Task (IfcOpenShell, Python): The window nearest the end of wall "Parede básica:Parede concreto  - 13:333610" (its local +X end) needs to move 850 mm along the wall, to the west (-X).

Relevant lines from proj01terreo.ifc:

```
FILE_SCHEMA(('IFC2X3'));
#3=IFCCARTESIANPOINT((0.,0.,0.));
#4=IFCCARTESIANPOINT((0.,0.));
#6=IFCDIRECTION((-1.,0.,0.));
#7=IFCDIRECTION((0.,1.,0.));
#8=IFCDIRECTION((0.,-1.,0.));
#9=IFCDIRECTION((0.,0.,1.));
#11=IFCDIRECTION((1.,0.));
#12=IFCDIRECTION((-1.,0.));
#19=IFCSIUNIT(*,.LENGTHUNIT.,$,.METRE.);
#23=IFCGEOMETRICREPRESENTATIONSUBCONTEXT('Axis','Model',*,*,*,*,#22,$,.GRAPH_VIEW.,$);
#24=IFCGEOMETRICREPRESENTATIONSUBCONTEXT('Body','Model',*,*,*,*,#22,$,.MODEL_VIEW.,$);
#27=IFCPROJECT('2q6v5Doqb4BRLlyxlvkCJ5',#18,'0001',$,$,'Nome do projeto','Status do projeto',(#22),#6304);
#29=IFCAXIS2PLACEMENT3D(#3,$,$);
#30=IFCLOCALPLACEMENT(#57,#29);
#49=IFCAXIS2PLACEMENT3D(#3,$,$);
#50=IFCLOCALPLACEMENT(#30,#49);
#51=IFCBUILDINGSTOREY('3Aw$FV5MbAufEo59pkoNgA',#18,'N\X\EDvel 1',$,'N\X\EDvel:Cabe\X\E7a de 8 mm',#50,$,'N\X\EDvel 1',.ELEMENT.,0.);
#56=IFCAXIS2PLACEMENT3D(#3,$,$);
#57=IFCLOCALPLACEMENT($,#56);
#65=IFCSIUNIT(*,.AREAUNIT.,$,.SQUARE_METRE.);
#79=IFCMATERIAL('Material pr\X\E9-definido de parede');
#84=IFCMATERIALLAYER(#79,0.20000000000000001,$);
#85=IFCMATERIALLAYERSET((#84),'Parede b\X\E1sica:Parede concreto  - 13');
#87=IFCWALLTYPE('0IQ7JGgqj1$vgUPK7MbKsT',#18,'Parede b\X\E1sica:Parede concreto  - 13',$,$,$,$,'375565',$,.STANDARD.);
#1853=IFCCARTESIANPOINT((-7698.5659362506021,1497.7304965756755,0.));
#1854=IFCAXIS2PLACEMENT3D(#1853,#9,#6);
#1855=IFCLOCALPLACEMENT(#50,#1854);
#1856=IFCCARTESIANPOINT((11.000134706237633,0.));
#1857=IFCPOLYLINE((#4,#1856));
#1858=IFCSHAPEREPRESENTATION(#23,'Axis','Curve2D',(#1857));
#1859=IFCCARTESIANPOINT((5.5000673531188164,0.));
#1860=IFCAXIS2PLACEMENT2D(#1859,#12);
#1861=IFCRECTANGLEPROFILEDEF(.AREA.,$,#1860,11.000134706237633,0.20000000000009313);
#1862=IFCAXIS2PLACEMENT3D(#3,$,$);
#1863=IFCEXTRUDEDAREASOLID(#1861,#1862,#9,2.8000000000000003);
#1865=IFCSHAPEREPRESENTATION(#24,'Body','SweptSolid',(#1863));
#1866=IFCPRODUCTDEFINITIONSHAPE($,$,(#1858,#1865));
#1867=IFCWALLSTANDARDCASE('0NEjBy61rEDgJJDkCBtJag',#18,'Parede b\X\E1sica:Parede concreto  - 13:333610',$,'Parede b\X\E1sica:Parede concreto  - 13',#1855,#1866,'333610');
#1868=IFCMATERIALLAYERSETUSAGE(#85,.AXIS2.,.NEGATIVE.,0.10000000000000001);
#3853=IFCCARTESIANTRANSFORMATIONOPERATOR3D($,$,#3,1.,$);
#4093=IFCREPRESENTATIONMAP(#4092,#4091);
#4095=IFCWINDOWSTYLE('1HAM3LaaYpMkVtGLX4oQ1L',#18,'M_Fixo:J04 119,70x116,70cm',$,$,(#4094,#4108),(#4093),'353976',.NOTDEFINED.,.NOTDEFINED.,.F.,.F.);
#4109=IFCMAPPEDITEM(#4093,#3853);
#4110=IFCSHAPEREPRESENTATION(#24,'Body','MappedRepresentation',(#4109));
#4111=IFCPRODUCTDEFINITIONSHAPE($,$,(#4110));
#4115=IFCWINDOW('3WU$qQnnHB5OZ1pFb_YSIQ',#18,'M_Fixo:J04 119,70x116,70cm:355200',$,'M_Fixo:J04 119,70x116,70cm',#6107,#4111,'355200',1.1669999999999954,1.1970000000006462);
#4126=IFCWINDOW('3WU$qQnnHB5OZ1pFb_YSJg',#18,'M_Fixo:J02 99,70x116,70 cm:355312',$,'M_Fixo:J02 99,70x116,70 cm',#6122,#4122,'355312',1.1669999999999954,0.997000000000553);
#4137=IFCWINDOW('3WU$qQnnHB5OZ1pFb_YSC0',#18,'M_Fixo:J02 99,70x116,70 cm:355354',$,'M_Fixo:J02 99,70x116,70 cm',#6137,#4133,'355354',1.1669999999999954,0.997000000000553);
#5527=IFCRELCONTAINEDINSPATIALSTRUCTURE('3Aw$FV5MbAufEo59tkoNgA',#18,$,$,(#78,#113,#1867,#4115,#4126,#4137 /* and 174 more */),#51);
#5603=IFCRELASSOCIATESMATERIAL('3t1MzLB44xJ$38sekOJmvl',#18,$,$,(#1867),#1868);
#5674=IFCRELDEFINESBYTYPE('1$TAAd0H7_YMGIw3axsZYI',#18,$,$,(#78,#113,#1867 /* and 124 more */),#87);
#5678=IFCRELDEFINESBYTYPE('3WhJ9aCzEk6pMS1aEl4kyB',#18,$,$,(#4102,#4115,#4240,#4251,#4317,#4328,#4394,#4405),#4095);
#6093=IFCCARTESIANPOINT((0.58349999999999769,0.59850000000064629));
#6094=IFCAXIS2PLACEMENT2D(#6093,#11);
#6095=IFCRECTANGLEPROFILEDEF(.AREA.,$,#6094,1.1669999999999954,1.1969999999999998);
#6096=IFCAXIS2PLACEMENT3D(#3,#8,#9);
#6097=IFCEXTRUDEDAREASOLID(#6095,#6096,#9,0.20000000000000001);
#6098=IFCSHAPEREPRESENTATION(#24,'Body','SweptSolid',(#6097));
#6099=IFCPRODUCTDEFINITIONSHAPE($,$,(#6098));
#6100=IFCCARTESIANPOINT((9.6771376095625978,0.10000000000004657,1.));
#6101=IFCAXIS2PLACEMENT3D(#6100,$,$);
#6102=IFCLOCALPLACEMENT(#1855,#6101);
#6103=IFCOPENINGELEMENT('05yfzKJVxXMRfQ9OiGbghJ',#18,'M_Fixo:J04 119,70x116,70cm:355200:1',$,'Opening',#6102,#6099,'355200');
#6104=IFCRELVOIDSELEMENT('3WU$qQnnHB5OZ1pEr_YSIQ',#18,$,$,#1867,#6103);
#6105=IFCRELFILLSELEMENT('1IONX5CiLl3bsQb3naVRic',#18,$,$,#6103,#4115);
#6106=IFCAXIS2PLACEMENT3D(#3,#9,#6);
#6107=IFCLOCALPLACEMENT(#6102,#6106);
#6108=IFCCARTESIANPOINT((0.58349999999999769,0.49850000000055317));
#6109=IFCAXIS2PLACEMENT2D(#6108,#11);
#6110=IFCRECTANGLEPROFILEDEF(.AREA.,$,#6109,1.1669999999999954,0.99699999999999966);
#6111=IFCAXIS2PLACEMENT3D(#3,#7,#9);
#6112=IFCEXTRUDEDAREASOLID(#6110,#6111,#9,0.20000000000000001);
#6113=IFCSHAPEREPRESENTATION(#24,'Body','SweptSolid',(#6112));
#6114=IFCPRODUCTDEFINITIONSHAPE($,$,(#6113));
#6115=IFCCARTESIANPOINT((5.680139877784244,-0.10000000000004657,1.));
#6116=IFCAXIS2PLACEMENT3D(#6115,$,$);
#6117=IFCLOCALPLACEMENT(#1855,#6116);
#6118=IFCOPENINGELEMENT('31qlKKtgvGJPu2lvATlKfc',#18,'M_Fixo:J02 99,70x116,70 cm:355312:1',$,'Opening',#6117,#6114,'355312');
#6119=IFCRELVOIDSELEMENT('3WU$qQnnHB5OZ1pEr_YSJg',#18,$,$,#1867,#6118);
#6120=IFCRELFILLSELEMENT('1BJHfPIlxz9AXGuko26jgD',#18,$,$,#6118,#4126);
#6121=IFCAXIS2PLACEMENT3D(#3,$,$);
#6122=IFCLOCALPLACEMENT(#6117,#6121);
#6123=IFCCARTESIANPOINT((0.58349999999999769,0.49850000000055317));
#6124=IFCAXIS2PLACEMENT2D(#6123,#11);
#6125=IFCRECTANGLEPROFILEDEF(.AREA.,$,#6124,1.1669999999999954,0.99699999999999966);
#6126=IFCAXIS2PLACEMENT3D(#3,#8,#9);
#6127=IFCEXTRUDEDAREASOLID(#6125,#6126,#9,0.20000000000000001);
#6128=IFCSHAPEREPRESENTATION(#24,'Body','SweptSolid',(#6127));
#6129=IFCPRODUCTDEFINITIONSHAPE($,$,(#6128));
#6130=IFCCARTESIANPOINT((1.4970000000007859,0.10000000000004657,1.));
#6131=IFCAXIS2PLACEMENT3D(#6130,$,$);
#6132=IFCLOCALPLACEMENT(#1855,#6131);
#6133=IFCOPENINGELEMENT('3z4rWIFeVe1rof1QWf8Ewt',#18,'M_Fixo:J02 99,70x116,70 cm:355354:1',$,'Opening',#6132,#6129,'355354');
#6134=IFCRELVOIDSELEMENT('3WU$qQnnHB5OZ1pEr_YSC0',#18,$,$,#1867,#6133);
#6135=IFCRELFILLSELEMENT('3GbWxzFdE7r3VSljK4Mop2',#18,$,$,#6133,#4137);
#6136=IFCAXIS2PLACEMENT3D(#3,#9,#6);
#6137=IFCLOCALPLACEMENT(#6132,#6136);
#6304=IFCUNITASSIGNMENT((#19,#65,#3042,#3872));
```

```python
import ifcopenshell
import ifcopenshell.api.geometry
import ifcopenshell.util.placement
import ifcopenshell.util.unit

model = ifcopenshell.open("proj01terreo.ifc")
unit_scale = ifcopenshell.util.unit.calculate_unit_scale(model)

window = model.by_guid("3WU$qQnnHB5OZ1pFb_YSIQ")
opening = window.FillsVoids[0].RelatingOpeningElement
wall = opening.VoidsElements[0].RelatingBuildingElement

wall_matrix = ifcopenshell.util.placement.get_local_placement(wall.ObjectPlacement)
shift = wall_matrix[:3, 0] * 0.85 / unit_scale
before = ifcopenshell.util.placement.get_local_placement(window.ObjectPlacement)[:3, 3].copy()

# The window is placed relative to its opening, so it follows when the opening moves.
matrix = ifcopenshell.util.placement.get_local_placement(opening.ObjectPlacement)
matrix[:3, 3] += shift
ifcopenshell.api.geometry.edit_object_placement(
    model, product=opening, matrix=matrix, is_si=False, should_transform_children=True
)

after = ifcopenshell.util.placement.get_local_placement(window.ObjectPlacement)[:3, 3]
print("window moved by", (after - before).round(3) + 0.0)

model.write("proj01terreo-out.ifc")
```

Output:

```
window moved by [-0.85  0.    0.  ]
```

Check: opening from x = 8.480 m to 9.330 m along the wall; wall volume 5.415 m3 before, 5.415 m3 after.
